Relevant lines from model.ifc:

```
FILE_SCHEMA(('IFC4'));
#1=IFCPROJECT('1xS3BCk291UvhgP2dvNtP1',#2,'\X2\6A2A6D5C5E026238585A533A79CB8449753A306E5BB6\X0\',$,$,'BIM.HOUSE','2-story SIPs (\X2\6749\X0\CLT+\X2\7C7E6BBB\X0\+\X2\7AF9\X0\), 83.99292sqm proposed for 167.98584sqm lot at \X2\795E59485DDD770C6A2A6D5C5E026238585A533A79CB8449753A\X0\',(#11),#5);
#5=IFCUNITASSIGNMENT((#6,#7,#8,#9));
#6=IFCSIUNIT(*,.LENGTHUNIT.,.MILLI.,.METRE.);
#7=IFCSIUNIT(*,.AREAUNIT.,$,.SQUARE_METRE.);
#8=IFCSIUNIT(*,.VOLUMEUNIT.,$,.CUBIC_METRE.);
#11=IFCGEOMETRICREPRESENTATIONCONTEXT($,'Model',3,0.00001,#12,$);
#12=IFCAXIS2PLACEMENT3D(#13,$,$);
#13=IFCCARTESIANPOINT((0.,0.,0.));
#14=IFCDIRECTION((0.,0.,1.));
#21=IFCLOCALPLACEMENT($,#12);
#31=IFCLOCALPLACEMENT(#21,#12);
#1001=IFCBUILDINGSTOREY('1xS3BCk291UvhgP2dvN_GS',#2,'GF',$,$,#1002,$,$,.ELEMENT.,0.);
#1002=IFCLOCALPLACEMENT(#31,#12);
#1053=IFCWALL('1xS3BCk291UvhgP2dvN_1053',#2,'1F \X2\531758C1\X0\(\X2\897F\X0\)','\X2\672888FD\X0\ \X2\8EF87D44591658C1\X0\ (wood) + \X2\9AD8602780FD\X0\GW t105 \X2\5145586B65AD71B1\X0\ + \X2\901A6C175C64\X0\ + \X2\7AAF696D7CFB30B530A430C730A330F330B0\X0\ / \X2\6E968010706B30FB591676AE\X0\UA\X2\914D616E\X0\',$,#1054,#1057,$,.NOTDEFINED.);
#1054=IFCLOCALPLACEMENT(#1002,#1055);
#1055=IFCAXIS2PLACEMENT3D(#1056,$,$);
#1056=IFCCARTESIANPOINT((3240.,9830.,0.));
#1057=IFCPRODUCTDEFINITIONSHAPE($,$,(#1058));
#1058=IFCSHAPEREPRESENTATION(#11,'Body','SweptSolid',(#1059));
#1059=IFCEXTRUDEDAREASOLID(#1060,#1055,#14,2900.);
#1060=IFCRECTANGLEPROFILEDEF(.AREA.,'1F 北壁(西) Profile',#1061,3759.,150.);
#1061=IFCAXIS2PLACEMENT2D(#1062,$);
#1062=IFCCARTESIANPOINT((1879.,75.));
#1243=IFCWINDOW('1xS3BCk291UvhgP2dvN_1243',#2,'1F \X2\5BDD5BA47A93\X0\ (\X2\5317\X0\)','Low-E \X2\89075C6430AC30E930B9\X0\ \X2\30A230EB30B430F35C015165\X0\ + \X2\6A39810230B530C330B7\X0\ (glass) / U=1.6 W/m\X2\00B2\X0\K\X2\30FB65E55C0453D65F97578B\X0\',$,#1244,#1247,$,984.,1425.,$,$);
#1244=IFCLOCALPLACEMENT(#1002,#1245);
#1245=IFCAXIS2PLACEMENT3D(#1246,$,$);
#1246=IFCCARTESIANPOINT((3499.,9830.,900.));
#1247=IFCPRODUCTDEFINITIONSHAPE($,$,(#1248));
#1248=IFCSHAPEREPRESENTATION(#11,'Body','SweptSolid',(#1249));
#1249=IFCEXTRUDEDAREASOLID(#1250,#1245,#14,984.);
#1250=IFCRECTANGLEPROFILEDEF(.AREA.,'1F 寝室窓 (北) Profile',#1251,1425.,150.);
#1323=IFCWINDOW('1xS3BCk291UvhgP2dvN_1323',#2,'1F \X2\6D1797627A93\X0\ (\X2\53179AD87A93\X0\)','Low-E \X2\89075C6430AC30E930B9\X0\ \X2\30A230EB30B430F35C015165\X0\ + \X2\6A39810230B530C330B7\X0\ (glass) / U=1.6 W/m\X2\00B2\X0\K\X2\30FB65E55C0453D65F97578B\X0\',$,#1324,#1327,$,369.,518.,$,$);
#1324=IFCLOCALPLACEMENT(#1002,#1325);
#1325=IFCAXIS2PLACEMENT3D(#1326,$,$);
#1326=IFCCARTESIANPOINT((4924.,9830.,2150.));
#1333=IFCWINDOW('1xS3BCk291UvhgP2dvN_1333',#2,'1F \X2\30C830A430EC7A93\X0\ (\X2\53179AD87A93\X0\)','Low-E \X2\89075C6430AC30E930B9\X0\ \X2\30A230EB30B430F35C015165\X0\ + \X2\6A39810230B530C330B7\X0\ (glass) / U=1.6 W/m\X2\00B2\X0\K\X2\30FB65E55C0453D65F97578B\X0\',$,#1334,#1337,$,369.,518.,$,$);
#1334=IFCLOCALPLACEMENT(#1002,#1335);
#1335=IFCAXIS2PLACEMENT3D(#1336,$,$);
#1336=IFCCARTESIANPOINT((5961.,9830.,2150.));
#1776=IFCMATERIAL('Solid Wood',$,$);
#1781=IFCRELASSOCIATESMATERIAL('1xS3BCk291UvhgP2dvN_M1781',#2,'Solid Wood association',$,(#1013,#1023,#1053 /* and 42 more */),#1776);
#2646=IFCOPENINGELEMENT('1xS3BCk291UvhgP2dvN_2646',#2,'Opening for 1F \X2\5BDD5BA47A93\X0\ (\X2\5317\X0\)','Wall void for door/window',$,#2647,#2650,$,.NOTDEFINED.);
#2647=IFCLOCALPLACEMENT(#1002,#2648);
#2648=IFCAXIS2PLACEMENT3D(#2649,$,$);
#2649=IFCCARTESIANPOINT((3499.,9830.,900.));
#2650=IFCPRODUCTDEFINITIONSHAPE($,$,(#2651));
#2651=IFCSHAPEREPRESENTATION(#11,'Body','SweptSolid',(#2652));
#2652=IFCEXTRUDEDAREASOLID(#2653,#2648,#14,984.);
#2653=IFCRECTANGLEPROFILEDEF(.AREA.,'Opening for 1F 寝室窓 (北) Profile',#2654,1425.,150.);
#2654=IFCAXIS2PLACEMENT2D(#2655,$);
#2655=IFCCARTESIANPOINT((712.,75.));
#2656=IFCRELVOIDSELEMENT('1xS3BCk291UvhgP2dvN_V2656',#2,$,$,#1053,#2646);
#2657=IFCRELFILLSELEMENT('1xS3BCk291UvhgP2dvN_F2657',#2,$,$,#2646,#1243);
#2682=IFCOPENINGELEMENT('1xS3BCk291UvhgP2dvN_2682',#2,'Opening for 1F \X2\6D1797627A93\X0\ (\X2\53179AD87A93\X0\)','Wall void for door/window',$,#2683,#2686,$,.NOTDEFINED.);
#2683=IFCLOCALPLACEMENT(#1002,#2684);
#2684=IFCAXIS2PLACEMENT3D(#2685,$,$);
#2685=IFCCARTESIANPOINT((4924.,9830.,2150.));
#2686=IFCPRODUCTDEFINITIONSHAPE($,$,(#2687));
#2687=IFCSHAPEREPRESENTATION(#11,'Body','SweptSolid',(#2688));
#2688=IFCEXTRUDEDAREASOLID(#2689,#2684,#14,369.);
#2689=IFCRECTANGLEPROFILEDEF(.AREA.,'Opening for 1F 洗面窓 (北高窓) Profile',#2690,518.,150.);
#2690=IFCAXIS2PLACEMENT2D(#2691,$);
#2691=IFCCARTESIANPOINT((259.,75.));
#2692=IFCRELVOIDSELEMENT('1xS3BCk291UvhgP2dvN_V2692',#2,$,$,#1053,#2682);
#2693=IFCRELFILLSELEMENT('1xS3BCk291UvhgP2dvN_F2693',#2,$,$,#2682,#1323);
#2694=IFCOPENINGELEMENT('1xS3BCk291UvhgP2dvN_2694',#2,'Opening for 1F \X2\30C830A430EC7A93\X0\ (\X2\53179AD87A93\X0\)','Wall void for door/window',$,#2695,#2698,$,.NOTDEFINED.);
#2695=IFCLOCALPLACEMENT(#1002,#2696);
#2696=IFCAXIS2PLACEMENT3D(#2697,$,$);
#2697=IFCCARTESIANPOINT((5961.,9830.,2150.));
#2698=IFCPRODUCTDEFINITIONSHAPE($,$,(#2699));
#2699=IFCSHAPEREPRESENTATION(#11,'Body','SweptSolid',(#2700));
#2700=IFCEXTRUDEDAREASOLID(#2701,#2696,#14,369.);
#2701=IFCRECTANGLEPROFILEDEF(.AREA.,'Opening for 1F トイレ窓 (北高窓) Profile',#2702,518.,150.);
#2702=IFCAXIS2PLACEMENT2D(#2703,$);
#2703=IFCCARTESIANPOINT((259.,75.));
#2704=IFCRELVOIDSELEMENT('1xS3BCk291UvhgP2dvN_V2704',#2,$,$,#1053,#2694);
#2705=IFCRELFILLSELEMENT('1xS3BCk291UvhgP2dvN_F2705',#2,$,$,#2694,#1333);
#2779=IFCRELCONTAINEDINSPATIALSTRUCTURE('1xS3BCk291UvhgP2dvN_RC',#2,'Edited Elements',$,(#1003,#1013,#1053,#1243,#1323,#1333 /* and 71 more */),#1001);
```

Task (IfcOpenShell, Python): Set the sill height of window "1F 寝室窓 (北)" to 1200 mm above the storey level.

```python
import numpy as np
import ifcopenshell
import ifcopenshell.api.geometry
import ifcopenshell.geom
import ifcopenshell.util.element
import ifcopenshell.util.placement
import ifcopenshell.util.shape
import ifcopenshell.util.unit

model = ifcopenshell.open("model.ifc")
unit_scale = ifcopenshell.util.unit.calculate_unit_scale(model)

window = model.by_guid("1xS3BCk291UvhgP2dvN_1243")
opening = window.FillsVoids[0].RelatingOpeningElement
storey = ifcopenshell.util.element.get_container(window, ifc_class="IfcBuildingStorey")
level = ifcopenshell.util.placement.get_local_placement(storey.ObjectPlacement)[2, 3]

# The opening's origin need not be at the sill, so measure its lowest point.
shape = ifcopenshell.geom.create_shape(ifcopenshell.geom.settings(), opening)
bottom = ifcopenshell.util.shape.get_shape_bottom_elevation(shape, shape.geometry) / unit_scale
dz = level + 1200.0 - bottom

shift = np.array([0.0, 0.0, dz])
# The window is not placed relative to its opening, so move both.
for product in (opening, window):
    matrix = ifcopenshell.util.placement.get_local_placement(product.ObjectPlacement)
    matrix[:3, 3] += shift
    ifcopenshell.api.geometry.edit_object_placement(model, product=product, matrix=matrix, is_si=False)

print(f"moved by {dz * unit_scale:+.3f} m")

model.write("model_v2.ifc")
```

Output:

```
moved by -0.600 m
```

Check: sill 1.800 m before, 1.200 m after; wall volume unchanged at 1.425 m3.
